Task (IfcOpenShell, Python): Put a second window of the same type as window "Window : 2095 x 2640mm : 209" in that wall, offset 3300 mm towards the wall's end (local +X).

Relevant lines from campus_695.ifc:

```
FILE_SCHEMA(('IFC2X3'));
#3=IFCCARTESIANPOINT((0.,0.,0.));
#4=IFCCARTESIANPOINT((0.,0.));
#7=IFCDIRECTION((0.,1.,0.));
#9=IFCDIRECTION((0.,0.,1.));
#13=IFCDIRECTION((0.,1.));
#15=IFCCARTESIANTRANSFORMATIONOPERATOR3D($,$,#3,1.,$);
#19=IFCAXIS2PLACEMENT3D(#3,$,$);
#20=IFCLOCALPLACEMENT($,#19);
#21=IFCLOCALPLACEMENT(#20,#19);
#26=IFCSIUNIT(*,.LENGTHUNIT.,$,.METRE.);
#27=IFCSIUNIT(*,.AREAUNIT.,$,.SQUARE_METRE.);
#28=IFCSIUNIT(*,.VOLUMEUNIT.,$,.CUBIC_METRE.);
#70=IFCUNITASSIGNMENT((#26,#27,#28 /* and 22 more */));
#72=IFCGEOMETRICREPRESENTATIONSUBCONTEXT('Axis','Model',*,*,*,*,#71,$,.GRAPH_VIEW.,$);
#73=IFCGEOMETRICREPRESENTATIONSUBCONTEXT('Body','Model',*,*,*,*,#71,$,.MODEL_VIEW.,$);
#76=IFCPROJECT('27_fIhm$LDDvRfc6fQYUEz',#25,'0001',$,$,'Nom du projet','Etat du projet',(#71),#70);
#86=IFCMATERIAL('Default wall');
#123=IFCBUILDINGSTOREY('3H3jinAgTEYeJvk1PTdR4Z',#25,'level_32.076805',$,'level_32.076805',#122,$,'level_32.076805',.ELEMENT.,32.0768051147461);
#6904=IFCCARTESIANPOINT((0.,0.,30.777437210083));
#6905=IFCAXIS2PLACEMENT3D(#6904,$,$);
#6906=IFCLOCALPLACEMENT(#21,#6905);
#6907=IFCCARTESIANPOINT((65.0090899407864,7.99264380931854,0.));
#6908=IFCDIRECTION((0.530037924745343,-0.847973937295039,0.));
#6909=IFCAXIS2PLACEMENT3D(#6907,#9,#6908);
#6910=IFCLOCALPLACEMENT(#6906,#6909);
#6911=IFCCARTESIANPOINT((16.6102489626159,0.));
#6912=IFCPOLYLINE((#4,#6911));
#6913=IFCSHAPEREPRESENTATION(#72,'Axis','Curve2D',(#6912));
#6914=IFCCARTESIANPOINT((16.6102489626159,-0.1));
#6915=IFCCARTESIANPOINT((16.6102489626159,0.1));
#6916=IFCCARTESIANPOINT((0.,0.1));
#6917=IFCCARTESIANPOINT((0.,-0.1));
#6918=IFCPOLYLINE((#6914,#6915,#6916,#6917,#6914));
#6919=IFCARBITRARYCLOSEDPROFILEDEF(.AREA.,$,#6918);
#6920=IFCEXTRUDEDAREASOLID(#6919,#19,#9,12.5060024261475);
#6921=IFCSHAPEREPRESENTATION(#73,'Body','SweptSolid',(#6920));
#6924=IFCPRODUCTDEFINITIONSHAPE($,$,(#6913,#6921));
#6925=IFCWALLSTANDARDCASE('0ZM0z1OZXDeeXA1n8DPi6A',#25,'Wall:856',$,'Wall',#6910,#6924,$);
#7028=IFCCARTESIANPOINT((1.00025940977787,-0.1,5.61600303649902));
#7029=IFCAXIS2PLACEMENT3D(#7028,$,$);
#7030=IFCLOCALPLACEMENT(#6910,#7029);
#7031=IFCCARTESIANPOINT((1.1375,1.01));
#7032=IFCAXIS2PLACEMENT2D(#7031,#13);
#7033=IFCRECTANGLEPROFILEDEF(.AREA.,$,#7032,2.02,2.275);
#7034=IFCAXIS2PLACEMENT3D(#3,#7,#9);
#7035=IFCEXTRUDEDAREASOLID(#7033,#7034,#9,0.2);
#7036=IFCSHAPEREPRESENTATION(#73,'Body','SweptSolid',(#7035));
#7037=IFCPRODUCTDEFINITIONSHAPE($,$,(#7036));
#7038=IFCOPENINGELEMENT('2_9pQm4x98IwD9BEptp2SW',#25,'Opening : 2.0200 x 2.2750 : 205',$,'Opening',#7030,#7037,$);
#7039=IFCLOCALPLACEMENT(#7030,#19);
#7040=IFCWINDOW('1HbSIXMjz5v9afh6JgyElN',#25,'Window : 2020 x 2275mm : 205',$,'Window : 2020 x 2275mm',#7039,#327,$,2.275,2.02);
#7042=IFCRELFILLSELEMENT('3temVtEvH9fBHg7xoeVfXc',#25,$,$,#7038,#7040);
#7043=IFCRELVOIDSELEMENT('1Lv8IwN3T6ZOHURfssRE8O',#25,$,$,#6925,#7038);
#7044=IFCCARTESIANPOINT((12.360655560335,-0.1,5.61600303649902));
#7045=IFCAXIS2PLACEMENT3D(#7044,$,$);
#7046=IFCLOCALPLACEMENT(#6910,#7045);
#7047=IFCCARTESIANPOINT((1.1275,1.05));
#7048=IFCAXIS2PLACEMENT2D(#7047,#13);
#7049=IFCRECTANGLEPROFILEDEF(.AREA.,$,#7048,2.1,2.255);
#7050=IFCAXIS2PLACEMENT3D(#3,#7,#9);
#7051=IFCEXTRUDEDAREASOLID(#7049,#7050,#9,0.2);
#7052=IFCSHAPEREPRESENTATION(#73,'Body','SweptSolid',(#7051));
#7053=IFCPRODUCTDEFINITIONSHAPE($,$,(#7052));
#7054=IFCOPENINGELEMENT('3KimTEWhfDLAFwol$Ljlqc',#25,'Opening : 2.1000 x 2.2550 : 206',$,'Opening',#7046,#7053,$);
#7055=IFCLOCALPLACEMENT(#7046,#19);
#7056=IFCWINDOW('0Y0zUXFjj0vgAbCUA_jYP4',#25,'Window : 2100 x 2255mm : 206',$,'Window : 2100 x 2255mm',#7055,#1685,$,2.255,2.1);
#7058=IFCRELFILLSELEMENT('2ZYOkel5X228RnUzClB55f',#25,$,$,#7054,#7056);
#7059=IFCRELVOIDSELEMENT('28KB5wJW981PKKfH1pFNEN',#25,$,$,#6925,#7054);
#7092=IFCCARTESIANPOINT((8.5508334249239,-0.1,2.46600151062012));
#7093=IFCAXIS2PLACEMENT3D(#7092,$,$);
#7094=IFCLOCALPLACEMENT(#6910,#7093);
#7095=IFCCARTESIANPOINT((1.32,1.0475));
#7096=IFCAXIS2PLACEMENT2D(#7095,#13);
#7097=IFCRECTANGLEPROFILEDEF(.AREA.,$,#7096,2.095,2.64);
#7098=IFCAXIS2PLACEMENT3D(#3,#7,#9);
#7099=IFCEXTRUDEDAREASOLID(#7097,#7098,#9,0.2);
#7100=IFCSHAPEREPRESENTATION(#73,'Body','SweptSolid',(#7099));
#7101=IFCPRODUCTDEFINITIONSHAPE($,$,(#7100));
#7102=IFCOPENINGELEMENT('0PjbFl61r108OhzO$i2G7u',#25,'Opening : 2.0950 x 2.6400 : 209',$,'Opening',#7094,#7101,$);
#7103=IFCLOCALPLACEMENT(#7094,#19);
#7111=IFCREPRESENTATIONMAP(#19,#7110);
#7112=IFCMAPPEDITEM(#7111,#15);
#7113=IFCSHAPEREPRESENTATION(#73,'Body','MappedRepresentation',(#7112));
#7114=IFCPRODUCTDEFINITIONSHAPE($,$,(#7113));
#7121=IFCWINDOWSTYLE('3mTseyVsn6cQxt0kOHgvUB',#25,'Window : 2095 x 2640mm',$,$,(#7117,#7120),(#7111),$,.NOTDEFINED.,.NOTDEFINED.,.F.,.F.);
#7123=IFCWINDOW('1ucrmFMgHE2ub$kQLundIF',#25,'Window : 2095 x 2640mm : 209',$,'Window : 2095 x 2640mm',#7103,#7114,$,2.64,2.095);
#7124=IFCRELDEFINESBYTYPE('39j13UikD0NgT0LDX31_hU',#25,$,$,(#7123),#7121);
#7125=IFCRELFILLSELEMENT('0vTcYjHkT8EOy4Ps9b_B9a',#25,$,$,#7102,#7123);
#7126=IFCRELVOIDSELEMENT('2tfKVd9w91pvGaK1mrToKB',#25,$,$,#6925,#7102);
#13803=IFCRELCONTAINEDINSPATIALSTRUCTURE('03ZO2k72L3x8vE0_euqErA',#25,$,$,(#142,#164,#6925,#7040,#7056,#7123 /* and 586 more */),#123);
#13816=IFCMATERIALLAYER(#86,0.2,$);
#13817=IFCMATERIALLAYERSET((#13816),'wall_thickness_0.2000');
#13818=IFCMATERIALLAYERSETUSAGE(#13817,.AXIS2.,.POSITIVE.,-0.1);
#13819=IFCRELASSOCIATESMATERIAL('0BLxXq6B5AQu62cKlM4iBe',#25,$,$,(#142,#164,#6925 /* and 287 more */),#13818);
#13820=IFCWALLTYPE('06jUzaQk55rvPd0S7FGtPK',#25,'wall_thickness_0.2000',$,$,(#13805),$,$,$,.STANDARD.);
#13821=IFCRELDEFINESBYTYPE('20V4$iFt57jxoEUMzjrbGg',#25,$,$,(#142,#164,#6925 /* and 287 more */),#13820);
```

```python
import ifcopenshell
import ifcopenshell.api.feature
import ifcopenshell.api.geometry
import ifcopenshell.api.root
import ifcopenshell.geom
import ifcopenshell.util.element
import ifcopenshell.util.placement
import ifcopenshell.util.shape
import ifcopenshell.util.unit

model = ifcopenshell.open("campus_695.ifc")
unit_scale = ifcopenshell.util.unit.calculate_unit_scale(model)
settings = ifcopenshell.geom.settings()


def volume(element):
    """Net volume in cubic metres, openings subtracted."""
    shape = ifcopenshell.geom.create_shape(settings, element)
    return ifcopenshell.util.shape.get_volume(shape.geometry)


window = model.by_guid("1ucrmFMgHE2ub$kQLundIF")
opening = window.FillsVoids[0].RelatingOpeningElement
wall = opening.VoidsElements[0].RelatingBuildingElement
before = volume(wall)
shift = ifcopenshell.util.placement.get_local_placement(wall.ObjectPlacement)[:3, 0] * 3.3 / unit_scale

# copy_class copies the void relationship, type, container and properties, but no geometry.
new_opening = ifcopenshell.api.root.copy_class(model, product=opening)
new_opening.Representation = ifcopenshell.util.element.copy_deep(
    model, opening.Representation, exclude=["IfcGeometricRepresentationContext", "IfcRepresentationMap"]
)
new_opening.Name = "Opening : 2.0950 x 2.6400"
new_window = ifcopenshell.api.root.copy_class(model, product=window)
new_window.Representation = ifcopenshell.util.element.copy_deep(
    model, window.Representation, exclude=["IfcGeometricRepresentationContext", "IfcRepresentationMap"]
)
new_window.Name = "Window : 2095 x 2640mm"
fills = ifcopenshell.api.feature.add_filling(model, opening=new_opening, element=new_window)
fills.OwnerHistory = new_window.OwnerHistory  # required in IFC2X3

for old, new in ((opening, new_opening), (window, new_window)):
    matrix = ifcopenshell.util.placement.get_local_placement(old.ObjectPlacement)
    matrix[:3, 3] += shift
    ifcopenshell.api.geometry.edit_object_placement(model, product=new, matrix=matrix, is_si=False)

after = volume(wall)

print(f"wall volume {before:.3f} -> {after:.3f} m3")

model.write("campus_695_updated.ifc")
```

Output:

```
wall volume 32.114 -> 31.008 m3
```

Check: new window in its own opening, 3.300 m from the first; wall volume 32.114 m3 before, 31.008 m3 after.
